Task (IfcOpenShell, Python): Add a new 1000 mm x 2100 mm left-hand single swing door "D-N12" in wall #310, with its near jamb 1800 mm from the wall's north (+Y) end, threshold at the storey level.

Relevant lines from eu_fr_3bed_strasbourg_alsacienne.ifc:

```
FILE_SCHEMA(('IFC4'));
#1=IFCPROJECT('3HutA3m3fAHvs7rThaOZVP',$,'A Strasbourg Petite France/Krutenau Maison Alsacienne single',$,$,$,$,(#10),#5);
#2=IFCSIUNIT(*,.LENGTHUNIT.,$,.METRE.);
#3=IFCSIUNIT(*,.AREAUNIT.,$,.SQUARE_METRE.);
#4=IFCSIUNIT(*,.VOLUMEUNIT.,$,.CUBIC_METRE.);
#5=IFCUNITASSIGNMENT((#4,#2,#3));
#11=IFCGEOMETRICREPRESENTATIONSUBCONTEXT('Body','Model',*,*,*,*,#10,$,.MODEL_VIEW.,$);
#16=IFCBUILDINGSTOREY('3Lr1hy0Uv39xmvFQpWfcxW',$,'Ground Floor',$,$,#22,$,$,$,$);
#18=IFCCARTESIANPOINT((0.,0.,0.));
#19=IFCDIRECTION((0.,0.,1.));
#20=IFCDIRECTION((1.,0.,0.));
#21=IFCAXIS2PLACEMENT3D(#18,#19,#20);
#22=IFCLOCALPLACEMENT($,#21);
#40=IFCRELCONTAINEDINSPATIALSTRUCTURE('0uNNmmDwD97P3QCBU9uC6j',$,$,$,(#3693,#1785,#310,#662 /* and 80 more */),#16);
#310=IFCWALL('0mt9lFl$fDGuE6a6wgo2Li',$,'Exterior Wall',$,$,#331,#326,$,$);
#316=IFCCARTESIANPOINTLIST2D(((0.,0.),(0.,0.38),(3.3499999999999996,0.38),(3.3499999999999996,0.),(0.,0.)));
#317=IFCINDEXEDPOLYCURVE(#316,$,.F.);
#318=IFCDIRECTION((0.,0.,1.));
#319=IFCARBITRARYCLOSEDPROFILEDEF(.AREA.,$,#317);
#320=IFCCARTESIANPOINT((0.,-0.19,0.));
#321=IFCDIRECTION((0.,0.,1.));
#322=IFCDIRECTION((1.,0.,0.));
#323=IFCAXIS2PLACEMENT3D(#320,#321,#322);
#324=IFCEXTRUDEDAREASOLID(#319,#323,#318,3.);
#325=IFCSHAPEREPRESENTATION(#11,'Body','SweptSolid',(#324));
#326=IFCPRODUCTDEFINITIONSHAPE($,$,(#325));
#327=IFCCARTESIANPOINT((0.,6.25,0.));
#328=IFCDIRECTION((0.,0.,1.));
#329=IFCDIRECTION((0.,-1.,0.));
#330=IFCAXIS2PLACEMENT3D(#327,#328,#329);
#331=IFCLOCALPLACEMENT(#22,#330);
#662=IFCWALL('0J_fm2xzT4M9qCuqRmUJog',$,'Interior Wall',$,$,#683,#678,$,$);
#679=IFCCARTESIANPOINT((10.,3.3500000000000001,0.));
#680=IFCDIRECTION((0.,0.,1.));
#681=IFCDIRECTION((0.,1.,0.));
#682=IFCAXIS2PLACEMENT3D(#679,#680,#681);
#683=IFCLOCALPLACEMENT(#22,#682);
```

```python
import numpy as np
import ifcopenshell
import ifcopenshell.api.feature
import ifcopenshell.api.geometry
import ifcopenshell.api.root
import ifcopenshell.api.spatial
import ifcopenshell.geom
import ifcopenshell.util.element
import ifcopenshell.util.placement
import ifcopenshell.util.representation
import ifcopenshell.util.shape
import ifcopenshell.util.unit

model = ifcopenshell.open("eu_fr_3bed_strasbourg_alsacienne.ifc")
unit_scale = ifcopenshell.util.unit.calculate_unit_scale(model)
settings = ifcopenshell.geom.settings()


def volume(element):
    """Net volume in cubic metres, openings subtracted."""
    shape = ifcopenshell.geom.create_shape(settings, element)
    return ifcopenshell.util.shape.get_volume(shape.geometry)


wall = model.by_id(310)
storey = ifcopenshell.util.element.get_container(wall, ifc_class="IfcBuildingStorey")
context = ifcopenshell.util.representation.get_context(model, "Model", "Body", "MODEL_VIEW")
before = volume(wall)

width, height, from_end, sill = 1, 2.1, 1.8, 0.0  # metres

# The wall runs along its own X axis, and the end named is its -X end.
wall_shape = ifcopenshell.geom.create_shape(settings, wall)
x, y, z = ifcopenshell.util.shape.get_vertices(wall_shape.geometry).T
start = x.min() + from_end
face, thickness = float(y.min()), float(y.max() - y.min())
wall_matrix = ifcopenshell.util.placement.get_local_placement(wall.ObjectPlacement)
level = ifcopenshell.util.placement.get_local_placement(storey.ObjectPlacement)[2, 3]


def in_wall(x, y):
    """Placement at x, y metres in the wall's axes, at sill height."""
    matrix = wall_matrix.copy()
    matrix[:, 3] = wall_matrix @ np.array([x / unit_scale, y / unit_scale, 0.0, 1.0])
    matrix[2, 3] = level + sill / unit_scale
    return matrix


# Opening: a box that overshoots both wall faces by 50 mm.
opening = ifcopenshell.api.root.create_entity(model, ifc_class="IfcOpeningElement", predefined_type="OPENING")
box = ifcopenshell.api.geometry.add_wall_representation(
    model, context=context, length=width, height=height, thickness=thickness + 0.1
)
ifcopenshell.api.geometry.assign_representation(model, product=opening, representation=box)
ifcopenshell.api.geometry.edit_object_placement(model, product=opening, matrix=in_wall(start, face - 0.05), is_si=False)
ifcopenshell.api.feature.add_feature(model, feature=opening, element=wall)

door = ifcopenshell.api.root.create_entity(model, ifc_class="IfcDoor", name="D-N12", predefined_type="DOOR")
door.OverallWidth, door.OverallHeight = width / unit_scale, height / unit_scale
door.OperationType = "SINGLE_SWING_LEFT"
body = ifcopenshell.api.geometry.add_door_representation(
    model,
    context=context,
    overall_width=door.OverallWidth,
    overall_height=door.OverallHeight,
    operation_type="SINGLE_SWING_LEFT",
    lining_properties={"LiningDepth": thickness / unit_scale, "ThresholdDepth": thickness / unit_scale},
)
ifcopenshell.api.geometry.assign_representation(model, product=door, representation=body)
ifcopenshell.api.spatial.assign_container(model, products=[door], relating_structure=storey)
ifcopenshell.api.feature.add_filling(model, opening=opening, element=door)

# The lining spans the wall, so the door starts at the wall face.
ifcopenshell.api.geometry.edit_object_placement(model, product=door, matrix=in_wall(start, face), is_si=False)

after = volume(wall)

print(f"wall volume {before:.3f} -> {after:.3f} m3")

model.write("eu_fr_3bed_strasbourg_alsacienne-out.ifc")
```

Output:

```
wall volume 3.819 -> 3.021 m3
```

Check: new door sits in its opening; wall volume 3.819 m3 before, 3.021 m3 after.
